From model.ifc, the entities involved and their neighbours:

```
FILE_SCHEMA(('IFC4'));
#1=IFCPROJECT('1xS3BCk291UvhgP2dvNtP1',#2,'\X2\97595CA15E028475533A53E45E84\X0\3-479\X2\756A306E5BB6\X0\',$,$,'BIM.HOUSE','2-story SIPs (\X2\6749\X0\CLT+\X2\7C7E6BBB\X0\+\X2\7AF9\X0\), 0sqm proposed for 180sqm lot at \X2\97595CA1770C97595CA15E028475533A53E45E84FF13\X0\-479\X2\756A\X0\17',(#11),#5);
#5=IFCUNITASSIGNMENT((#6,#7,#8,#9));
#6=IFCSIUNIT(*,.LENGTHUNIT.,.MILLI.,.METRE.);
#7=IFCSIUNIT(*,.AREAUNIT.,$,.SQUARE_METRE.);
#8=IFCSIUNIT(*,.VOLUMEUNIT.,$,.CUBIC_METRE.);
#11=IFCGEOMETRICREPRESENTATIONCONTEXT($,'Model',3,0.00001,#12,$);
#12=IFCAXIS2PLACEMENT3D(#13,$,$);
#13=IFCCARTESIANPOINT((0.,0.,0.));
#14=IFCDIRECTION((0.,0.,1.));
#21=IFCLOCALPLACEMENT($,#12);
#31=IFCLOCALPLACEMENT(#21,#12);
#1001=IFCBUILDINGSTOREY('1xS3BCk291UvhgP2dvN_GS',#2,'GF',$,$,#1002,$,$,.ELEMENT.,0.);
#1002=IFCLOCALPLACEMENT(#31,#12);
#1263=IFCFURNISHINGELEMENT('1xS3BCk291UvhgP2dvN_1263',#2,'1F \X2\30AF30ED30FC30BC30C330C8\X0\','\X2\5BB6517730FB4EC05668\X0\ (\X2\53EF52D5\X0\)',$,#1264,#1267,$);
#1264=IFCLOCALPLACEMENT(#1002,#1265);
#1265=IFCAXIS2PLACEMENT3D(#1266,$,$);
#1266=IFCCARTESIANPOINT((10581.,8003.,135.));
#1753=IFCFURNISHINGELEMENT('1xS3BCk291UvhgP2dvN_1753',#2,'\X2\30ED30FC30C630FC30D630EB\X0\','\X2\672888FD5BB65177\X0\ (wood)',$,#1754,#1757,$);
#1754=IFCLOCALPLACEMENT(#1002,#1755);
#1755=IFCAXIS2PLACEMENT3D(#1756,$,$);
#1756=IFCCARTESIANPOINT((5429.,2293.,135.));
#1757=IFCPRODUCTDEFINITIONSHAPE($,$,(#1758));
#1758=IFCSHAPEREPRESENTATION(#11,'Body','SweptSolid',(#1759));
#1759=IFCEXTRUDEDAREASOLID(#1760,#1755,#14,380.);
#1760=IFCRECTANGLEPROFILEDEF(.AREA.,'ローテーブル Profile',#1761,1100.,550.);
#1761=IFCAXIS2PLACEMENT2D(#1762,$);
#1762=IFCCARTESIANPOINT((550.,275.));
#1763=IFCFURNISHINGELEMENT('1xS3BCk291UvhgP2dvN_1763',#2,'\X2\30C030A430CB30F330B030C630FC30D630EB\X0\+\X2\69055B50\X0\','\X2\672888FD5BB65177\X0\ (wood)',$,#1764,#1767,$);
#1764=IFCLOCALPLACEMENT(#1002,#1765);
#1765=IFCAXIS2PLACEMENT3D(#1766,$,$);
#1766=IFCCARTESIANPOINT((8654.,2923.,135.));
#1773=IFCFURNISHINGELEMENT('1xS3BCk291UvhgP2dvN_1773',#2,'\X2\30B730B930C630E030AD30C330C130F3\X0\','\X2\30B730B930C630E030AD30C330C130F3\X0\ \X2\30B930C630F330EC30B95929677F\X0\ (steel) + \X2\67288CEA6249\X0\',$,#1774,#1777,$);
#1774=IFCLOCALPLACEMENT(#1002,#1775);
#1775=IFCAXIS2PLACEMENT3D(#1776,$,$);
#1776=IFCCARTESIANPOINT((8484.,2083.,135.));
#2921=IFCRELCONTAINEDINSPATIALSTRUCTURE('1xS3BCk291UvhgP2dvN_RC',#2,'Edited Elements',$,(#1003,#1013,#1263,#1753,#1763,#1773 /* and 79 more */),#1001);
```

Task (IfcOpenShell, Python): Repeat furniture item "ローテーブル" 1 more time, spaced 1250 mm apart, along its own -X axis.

```python
import ifcopenshell
import ifcopenshell.api.geometry
import ifcopenshell.api.root
import ifcopenshell.util.element
import ifcopenshell.util.placement
import ifcopenshell.util.unit

model = ifcopenshell.open("model.ifc")
unit_scale = ifcopenshell.util.unit.calculate_unit_scale(model)


def reuse_history(source, copy):
    """copy_class also copies each property set's owner history, people and application; keep the originals."""
    for rel in copy.IsDefinedBy:
        if rel.is_a("IfcRelDefinesByProperties") and (history := rel.RelatingPropertyDefinition.OwnerHistory):
            rel.RelatingPropertyDefinition.OwnerHistory = source.OwnerHistory
            ifcopenshell.util.element.remove_deep2(model, history)


source = model.by_guid("1xS3BCk291UvhgP2dvN_1753")
base = ifcopenshell.util.placement.get_local_placement(source.ObjectPlacement)
step = -base[:3, 0] * 1.25 / unit_scale

for i in range(1, 2):
    copy = ifcopenshell.api.root.copy_class(model, product=source)
    copy.Representation = ifcopenshell.util.element.copy_deep(
        model, source.Representation, exclude=["IfcGeometricRepresentationContext", "IfcRepresentationMap"]
    )
    reuse_history(source, copy)
    matrix = base.copy()
    matrix[:3, 3] += i * step
    print("added at", matrix[:3, 3].round(3) + 0.0)
    ifcopenshell.api.geometry.edit_object_placement(model, product=copy, matrix=matrix, is_si=False)

model.write("model_updated.ifc")
```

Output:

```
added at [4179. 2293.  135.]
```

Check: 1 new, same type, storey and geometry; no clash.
